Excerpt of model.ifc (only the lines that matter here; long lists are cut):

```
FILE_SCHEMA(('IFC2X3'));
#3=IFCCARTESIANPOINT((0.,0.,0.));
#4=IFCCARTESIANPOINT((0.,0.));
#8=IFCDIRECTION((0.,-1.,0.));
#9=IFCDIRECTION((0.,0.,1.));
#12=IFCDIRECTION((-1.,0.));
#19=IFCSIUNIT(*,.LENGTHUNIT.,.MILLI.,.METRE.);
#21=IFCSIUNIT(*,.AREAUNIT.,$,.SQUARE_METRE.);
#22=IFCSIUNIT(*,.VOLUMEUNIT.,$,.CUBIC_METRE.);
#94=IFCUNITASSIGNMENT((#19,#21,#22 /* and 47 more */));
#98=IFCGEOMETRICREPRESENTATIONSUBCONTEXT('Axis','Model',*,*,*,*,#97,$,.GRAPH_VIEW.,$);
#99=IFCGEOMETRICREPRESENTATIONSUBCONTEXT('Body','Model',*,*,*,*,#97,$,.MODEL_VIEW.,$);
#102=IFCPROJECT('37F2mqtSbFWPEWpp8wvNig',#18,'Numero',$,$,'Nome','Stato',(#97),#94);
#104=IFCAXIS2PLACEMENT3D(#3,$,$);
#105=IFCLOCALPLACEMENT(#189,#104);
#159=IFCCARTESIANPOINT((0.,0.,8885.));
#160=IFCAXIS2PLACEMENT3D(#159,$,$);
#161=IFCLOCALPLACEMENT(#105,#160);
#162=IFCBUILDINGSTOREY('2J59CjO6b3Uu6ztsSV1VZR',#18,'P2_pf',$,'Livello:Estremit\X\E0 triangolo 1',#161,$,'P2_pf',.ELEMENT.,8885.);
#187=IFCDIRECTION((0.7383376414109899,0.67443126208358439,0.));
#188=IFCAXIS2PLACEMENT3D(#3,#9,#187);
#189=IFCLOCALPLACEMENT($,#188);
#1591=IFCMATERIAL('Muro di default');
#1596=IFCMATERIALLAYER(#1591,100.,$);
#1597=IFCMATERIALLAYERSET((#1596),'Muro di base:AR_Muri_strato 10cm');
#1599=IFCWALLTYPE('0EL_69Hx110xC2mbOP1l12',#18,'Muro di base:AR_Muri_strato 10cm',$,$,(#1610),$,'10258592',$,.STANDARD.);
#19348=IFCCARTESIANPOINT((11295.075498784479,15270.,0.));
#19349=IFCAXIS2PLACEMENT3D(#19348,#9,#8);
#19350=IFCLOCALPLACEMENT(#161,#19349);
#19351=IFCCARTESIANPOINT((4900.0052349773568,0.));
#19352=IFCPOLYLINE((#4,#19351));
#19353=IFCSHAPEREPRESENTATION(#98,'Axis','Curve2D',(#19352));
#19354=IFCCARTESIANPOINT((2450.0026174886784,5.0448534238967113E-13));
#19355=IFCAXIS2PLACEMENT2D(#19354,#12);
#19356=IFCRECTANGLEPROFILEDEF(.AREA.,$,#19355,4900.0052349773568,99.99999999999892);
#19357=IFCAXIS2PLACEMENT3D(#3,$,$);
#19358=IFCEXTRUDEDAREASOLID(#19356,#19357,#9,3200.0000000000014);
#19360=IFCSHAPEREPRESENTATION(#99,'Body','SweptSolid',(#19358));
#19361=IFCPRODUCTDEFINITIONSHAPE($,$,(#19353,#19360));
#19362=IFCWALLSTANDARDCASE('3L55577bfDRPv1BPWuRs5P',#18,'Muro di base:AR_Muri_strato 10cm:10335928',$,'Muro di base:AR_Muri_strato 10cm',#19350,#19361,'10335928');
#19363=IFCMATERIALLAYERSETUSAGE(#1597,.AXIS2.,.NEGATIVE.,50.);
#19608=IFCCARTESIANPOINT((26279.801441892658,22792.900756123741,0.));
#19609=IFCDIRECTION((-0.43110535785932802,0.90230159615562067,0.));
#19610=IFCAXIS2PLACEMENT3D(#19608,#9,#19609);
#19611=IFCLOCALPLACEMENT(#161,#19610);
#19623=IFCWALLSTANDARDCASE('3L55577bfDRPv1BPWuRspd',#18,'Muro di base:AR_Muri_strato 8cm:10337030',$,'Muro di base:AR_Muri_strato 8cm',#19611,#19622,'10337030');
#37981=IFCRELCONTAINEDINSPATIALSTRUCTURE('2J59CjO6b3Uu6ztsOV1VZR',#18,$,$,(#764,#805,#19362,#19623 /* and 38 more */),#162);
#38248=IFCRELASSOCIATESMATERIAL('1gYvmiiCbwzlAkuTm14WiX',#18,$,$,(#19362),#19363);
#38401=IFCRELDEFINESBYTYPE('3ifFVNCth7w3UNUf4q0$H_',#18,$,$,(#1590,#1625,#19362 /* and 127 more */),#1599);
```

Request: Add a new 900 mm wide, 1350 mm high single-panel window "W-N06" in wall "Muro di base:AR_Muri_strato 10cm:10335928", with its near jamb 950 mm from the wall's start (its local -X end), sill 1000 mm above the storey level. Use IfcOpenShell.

```python
import numpy as np
import ifcopenshell
import ifcopenshell.api.feature
import ifcopenshell.api.geometry
import ifcopenshell.api.root
import ifcopenshell.api.spatial
import ifcopenshell.api.type
import ifcopenshell.geom
import ifcopenshell.util.element
import ifcopenshell.util.placement
import ifcopenshell.util.representation
import ifcopenshell.util.shape
import ifcopenshell.util.unit

model = ifcopenshell.open("model.ifc")
unit_scale = ifcopenshell.util.unit.calculate_unit_scale(model)
settings = ifcopenshell.geom.settings()


def volume(element):
    """Net volume in cubic metres, openings subtracted."""
    shape = ifcopenshell.geom.create_shape(settings, element)
    return ifcopenshell.util.shape.get_volume(shape.geometry)


wall = model.by_guid("3L55577bfDRPv1BPWuRs5P")
storey = ifcopenshell.util.element.get_container(wall, ifc_class="IfcBuildingStorey")
context = ifcopenshell.util.representation.get_context(model, "Model", "Body", "MODEL_VIEW")
before = volume(wall)

width, height, from_end, sill = 0.9, 1.35, 0.95, 1  # metres

# The wall runs along its own X axis, and the end named is its -X end.
wall_shape = ifcopenshell.geom.create_shape(settings, wall)
x, y, z = ifcopenshell.util.shape.get_vertices(wall_shape.geometry).T
start = x.min() + from_end
face, thickness = float(y.min()), float(y.max() - y.min())
wall_matrix = ifcopenshell.util.placement.get_local_placement(wall.ObjectPlacement)
level = ifcopenshell.util.placement.get_local_placement(storey.ObjectPlacement)[2, 3]


def in_wall(x, y):
    """Placement at x, y metres in the wall's axes, at sill height."""
    matrix = wall_matrix.copy()
    matrix[:, 3] = wall_matrix @ np.array([x / unit_scale, y / unit_scale, 0.0, 1.0])
    matrix[2, 3] = level + sill / unit_scale
    return matrix


# Opening: a box that overshoots both wall faces by 50 mm.
opening = ifcopenshell.api.root.create_entity(model, ifc_class="IfcOpeningElement")
box = ifcopenshell.api.geometry.add_wall_representation(
    model, context=context, length=width, height=height, thickness=thickness + 0.1
)
ifcopenshell.api.geometry.assign_representation(model, product=opening, representation=box)
ifcopenshell.api.geometry.edit_object_placement(model, product=opening, matrix=in_wall(start, face - 0.05), is_si=False)
ifcopenshell.api.feature.add_feature(model, feature=opening, element=wall)

window = ifcopenshell.api.root.create_entity(model, ifc_class="IfcWindow", name="W-N06")
window.OverallWidth, window.OverallHeight = width / unit_scale, height / unit_scale
body = ifcopenshell.api.geometry.add_window_representation(
    model,
    context=context,
    overall_width=window.OverallWidth,
    overall_height=window.OverallHeight,
    partition_type="SINGLE_PANEL",
)
ifcopenshell.api.geometry.assign_representation(model, product=window, representation=body)
ifcopenshell.api.spatial.assign_container(model, products=[window], relating_structure=storey)
fills = ifcopenshell.api.feature.add_filling(model, opening=opening, element=window)
fills.OwnerHistory = window.OwnerHistory  # required in IFC2X3

# IFC2X3 keeps the operation on the window style.
style = ifcopenshell.api.root.create_entity(model, ifc_class="IfcWindowStyle", name="W-N06")
style.OperationType, style.ConstructionType = "SINGLE_PANEL", "NOTDEFINED"
style.ParameterTakesPrecedence = style.Sizeable = False
ifcopenshell.api.type.assign_type(model, related_objects=[window], relating_type=style)

# Centre the window in the wall's thickness.
ifcopenshell.api.geometry.edit_object_placement(model, product=window, matrix=in_wall(start, face), is_si=False)
window_shape = ifcopenshell.geom.create_shape(settings, window)
depth = ifcopenshell.util.shape.get_vertices(window_shape.geometry)[:, 1]
offset = face + thickness / 2 - (depth.min() + depth.max()) / 2
ifcopenshell.api.geometry.edit_object_placement(model, product=window, matrix=in_wall(start, offset), is_si=False)

after = volume(wall)

print(f"wall volume {before:.3f} -> {after:.3f} m3")

model.write("model_updated.ifc")
```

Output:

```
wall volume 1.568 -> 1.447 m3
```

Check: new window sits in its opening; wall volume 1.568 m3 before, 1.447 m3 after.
